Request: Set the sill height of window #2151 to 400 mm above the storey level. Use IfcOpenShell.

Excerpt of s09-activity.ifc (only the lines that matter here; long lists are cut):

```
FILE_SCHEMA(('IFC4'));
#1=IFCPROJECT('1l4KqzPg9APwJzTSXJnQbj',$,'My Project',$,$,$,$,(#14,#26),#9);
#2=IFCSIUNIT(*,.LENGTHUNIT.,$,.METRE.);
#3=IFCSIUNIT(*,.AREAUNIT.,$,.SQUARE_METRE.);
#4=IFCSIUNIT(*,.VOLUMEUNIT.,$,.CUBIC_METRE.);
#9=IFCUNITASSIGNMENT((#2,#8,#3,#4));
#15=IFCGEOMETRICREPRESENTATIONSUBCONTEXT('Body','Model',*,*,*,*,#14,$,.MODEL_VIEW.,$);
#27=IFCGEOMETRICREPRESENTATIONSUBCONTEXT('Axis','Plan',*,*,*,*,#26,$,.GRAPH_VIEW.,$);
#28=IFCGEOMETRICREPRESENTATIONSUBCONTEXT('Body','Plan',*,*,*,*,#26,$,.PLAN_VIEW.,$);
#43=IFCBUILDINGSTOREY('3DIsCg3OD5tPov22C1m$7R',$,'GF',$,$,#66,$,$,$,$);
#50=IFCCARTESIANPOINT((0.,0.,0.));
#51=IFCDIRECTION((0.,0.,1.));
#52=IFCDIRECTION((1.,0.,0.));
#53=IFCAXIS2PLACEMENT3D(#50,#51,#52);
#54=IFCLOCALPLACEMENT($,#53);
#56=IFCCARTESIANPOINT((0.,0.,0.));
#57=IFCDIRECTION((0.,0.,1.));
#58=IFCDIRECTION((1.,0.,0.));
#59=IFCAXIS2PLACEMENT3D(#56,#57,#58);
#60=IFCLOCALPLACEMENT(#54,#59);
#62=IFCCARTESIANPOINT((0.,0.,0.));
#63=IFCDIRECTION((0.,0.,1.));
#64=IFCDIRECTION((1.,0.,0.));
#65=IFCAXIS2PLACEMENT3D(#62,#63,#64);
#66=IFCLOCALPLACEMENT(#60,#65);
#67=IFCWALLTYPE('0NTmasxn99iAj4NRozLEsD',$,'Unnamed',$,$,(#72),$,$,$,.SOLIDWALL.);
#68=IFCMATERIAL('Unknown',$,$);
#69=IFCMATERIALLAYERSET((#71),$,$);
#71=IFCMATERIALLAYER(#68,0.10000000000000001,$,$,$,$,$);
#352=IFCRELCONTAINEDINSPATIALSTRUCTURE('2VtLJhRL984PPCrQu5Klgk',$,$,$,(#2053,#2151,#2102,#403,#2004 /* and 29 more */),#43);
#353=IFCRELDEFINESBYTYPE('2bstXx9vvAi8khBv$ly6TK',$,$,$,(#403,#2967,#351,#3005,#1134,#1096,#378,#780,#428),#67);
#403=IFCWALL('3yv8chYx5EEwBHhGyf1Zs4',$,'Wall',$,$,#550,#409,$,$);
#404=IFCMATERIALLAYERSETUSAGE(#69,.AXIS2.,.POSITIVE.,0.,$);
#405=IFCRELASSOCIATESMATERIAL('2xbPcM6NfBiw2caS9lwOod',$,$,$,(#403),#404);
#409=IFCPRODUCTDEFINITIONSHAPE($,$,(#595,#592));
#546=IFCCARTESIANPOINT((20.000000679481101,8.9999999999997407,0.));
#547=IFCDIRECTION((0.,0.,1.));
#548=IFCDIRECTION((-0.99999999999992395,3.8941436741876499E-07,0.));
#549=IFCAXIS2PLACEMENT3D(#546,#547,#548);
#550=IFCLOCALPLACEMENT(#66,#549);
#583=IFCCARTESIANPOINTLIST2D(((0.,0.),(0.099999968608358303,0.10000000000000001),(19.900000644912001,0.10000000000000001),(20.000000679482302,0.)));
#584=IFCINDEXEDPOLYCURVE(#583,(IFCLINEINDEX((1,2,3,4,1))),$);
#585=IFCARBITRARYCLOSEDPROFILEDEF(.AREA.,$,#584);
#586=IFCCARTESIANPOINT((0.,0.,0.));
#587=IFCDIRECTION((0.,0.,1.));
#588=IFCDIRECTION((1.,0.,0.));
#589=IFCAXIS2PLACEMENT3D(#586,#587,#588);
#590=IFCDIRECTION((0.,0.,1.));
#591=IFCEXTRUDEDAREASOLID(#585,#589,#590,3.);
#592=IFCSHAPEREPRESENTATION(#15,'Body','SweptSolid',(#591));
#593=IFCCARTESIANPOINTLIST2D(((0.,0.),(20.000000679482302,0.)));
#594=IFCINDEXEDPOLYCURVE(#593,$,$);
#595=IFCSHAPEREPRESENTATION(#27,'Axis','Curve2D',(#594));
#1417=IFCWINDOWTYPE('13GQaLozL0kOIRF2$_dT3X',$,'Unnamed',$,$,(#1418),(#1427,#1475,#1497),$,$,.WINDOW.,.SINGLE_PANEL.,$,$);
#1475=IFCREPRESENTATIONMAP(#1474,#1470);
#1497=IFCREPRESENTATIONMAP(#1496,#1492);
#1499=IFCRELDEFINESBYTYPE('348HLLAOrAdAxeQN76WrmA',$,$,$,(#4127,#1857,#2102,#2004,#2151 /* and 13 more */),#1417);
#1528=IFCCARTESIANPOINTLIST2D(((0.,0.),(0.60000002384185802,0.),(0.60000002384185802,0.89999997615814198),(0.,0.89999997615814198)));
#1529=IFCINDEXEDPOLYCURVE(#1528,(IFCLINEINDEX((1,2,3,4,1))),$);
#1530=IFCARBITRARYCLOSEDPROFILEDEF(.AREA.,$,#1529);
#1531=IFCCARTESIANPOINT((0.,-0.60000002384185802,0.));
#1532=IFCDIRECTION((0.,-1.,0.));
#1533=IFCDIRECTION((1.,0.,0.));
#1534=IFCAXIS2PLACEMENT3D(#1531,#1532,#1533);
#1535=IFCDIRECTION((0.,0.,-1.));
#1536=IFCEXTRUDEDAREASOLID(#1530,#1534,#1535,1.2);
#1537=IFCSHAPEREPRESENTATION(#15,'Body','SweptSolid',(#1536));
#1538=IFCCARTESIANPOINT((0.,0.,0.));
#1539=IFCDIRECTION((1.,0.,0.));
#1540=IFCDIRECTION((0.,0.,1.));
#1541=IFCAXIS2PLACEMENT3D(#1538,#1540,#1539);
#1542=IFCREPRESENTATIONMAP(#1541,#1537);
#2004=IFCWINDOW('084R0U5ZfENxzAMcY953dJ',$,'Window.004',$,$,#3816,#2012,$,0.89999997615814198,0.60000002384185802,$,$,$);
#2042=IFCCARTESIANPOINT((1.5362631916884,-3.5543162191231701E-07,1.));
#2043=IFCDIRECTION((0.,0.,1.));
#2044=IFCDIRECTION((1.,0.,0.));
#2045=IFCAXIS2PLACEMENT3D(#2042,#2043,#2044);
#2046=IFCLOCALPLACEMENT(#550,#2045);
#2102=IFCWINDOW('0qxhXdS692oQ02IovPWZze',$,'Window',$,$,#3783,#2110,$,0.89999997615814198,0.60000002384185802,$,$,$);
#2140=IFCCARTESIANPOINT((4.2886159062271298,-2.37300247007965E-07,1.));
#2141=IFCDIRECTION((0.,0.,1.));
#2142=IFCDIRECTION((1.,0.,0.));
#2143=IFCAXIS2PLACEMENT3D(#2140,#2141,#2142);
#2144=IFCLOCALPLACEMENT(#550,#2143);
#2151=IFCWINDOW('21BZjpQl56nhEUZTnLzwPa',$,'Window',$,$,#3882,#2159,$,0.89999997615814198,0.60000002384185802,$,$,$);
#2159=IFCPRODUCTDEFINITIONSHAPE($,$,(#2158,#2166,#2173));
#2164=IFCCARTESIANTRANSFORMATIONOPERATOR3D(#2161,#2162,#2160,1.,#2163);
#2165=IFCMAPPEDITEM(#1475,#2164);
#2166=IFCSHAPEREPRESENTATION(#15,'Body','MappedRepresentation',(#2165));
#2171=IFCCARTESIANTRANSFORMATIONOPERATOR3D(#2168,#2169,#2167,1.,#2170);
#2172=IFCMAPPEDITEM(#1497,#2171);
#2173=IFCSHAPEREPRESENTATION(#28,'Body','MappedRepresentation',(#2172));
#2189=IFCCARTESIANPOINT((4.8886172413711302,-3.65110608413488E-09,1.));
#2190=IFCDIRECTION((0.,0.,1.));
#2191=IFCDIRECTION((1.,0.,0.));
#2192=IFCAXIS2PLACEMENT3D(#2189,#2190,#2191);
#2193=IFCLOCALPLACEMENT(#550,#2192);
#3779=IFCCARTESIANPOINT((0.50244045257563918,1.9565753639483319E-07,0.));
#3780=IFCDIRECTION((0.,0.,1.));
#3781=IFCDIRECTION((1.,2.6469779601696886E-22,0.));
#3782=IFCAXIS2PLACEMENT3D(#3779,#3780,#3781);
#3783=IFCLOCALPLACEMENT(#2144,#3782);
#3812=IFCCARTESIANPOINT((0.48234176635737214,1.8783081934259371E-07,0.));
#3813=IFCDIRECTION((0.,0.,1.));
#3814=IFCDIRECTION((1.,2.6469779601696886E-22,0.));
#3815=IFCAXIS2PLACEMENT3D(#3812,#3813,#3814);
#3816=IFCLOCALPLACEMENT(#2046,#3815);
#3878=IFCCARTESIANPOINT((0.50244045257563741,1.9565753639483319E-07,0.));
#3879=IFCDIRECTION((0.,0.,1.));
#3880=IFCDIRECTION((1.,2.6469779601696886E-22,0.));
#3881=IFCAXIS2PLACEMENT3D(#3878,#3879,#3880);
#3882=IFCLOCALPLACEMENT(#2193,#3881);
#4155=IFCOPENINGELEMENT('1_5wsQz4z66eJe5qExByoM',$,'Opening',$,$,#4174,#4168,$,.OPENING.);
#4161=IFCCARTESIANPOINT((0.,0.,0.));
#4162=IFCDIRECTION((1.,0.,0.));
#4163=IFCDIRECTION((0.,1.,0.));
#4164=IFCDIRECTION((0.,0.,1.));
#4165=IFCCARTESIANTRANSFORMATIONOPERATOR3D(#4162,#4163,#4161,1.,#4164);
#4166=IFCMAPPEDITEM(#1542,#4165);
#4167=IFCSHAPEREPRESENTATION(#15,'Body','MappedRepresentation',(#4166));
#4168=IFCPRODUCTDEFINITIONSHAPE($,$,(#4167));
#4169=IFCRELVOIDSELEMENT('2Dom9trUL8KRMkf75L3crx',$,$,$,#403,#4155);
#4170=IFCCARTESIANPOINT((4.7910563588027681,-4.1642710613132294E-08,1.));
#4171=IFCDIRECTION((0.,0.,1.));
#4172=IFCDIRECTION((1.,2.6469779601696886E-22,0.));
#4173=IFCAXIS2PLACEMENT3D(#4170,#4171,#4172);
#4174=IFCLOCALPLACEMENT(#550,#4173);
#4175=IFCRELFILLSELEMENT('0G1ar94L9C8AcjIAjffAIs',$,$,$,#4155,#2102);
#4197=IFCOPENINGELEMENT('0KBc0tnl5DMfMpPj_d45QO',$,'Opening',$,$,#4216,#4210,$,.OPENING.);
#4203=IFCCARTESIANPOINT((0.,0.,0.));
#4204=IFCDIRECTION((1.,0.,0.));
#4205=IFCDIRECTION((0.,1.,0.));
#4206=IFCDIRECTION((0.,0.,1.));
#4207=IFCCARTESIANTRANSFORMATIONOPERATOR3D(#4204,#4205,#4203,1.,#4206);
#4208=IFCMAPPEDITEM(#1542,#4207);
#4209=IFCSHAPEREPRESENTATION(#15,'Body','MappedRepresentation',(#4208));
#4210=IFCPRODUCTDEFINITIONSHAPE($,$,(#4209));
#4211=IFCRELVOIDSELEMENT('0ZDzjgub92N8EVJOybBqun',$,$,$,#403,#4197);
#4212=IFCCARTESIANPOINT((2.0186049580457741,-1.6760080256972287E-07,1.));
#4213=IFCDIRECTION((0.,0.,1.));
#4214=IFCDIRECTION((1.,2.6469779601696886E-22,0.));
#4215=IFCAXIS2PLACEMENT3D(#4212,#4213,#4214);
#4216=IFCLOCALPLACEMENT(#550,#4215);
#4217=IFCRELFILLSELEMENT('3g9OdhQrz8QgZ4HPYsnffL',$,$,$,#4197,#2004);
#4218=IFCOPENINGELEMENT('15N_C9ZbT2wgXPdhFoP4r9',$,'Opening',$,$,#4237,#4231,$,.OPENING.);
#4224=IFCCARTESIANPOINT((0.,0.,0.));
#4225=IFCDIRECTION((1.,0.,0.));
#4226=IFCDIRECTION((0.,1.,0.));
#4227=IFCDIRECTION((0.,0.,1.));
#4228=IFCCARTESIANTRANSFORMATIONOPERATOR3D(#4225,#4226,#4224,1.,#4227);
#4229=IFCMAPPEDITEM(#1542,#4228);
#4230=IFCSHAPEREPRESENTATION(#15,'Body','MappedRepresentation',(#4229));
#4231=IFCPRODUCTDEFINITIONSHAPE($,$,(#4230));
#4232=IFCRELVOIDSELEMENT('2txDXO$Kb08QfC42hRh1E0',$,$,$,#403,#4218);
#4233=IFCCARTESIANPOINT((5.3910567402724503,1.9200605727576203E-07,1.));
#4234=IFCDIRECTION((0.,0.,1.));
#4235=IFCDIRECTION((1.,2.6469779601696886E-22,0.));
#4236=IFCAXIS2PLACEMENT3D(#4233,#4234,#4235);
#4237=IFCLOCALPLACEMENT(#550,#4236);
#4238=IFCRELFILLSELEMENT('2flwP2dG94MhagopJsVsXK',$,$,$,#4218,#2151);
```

```python
import numpy as np
import ifcopenshell
import ifcopenshell.api.geometry
import ifcopenshell.geom
import ifcopenshell.util.element
import ifcopenshell.util.placement
import ifcopenshell.util.shape
import ifcopenshell.util.unit

model = ifcopenshell.open("s09-activity.ifc")
unit_scale = ifcopenshell.util.unit.calculate_unit_scale(model)

window = model.by_id(2151)
opening = window.FillsVoids[0].RelatingOpeningElement
storey = ifcopenshell.util.element.get_container(window, ifc_class="IfcBuildingStorey")
level = ifcopenshell.util.placement.get_local_placement(storey.ObjectPlacement)[2, 3]

# The opening's origin need not be at the sill, so measure its lowest point.
shape = ifcopenshell.geom.create_shape(ifcopenshell.geom.settings(), opening)
bottom = ifcopenshell.util.shape.get_shape_bottom_elevation(shape, shape.geometry) / unit_scale
dz = level + 0.4 - bottom

shift = np.array([0.0, 0.0, dz])
# The window is not placed relative to its opening, so move both.
for product in (opening, window):
    matrix = ifcopenshell.util.placement.get_local_placement(product.ObjectPlacement)
    matrix[:3, 3] += shift
    ifcopenshell.api.geometry.edit_object_placement(model, product=product, matrix=matrix, is_si=False)

print(f"moved by {dz * unit_scale:+.3f} m")

model.write("s09-activity_rev.ifc")
```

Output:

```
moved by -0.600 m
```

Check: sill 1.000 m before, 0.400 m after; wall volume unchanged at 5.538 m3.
